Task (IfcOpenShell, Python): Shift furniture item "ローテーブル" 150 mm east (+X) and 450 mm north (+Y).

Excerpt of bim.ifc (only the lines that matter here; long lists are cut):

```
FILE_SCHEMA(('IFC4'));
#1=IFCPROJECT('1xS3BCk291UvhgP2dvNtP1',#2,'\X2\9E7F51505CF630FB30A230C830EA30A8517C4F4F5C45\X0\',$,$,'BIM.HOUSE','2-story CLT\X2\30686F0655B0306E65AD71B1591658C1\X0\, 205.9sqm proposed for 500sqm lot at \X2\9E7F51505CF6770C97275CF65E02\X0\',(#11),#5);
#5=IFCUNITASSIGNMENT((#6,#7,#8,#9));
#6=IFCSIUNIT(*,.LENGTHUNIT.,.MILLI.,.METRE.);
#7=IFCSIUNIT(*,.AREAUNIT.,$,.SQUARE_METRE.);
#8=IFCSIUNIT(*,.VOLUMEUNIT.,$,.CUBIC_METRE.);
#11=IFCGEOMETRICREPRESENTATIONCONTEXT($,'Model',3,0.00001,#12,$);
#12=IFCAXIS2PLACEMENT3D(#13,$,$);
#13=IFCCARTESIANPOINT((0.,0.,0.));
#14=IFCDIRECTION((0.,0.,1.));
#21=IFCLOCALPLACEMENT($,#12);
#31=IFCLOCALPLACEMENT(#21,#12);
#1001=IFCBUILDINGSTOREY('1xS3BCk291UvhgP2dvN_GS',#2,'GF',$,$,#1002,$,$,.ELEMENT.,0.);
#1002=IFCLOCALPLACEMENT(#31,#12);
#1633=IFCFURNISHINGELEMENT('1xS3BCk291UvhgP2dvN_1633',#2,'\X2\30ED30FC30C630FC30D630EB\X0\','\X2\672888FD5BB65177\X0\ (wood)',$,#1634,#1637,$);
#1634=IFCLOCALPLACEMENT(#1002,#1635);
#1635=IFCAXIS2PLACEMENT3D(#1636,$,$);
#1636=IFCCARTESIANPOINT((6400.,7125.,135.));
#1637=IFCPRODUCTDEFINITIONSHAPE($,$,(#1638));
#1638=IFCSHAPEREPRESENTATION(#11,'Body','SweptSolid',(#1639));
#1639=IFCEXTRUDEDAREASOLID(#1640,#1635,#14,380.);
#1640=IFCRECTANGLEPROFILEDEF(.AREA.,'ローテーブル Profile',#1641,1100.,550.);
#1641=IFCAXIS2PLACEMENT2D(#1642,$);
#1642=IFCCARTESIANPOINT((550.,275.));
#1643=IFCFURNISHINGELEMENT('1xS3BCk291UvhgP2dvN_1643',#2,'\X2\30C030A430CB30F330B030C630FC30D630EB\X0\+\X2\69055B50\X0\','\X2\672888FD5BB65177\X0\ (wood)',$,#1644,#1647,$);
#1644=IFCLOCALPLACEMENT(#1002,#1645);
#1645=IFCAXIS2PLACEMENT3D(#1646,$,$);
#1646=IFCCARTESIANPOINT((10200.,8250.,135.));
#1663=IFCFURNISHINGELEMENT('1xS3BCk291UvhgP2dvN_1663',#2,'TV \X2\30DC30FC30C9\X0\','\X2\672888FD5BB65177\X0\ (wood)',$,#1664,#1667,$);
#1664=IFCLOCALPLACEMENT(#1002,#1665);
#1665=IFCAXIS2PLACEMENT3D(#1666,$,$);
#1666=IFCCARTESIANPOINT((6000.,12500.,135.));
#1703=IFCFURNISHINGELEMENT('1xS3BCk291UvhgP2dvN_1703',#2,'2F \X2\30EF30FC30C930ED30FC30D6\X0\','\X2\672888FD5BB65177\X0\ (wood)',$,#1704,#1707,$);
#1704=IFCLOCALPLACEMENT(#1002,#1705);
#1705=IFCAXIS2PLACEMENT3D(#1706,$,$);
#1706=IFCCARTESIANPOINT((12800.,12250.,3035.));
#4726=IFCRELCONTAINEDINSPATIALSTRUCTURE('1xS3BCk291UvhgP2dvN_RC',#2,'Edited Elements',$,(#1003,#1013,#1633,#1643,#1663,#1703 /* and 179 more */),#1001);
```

```python
import ifcopenshell
import ifcopenshell.api.geometry
import ifcopenshell.util.placement
import ifcopenshell.util.unit

model = ifcopenshell.open("bim.ifc")
unit_scale = ifcopenshell.util.unit.calculate_unit_scale(model)

item = model.by_guid("1xS3BCk291UvhgP2dvN_1633")
matrix = ifcopenshell.util.placement.get_local_placement(item.ObjectPlacement)
matrix[0, 3] += 0.15 / unit_scale
matrix[1, 3] += 0.45 / unit_scale
ifcopenshell.api.geometry.edit_object_placement(model, product=item, matrix=matrix, is_si=False)

print(ifcopenshell.util.placement.get_local_placement(item.ObjectPlacement).round(3) + 0.0)

model.write("bim_updated.ifc")
```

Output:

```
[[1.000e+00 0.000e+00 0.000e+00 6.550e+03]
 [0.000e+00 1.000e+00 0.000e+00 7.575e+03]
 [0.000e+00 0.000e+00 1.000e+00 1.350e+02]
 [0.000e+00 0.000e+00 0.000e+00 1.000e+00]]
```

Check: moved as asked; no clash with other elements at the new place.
